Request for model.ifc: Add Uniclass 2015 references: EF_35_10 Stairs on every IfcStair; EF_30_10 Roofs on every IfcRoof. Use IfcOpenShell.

First a look at what the model holds.

```python
import ifcopenshell

model = ifcopenshell.open("model.ifc")
print(model.schema)
print("classifications:", [c.Name for c in model.by_type("IfcClassification")])
for ifc_class in ("IfcDoor", "IfcRoof", "IfcStair", "IfcWall", "IfcWindow"):
    print(ifc_class, len(model.by_type(ifc_class)))
```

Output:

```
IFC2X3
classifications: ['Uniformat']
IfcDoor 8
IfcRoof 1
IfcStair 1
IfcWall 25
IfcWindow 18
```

```python
import ifcopenshell
import ifcopenshell.api.classification

model = ifcopenshell.open("model.ifc")

# IFC2X3 requires Source and Edition and has no link from the project to the system.
system = model.create_entity("IfcClassification", Source="NBS", Edition="2015", Name="Uniclass 2015")

codes = {
    "IfcStair": ("EF_35_10", "Stairs"),
    "IfcRoof": ("EF_30_10", "Roofs"),
}
for ifc_class, (code, name) in codes.items():
    products = model.by_type(ifc_class)
    ifcopenshell.api.classification.add_reference(
        model, products=products, classification=system, identification=code, name=name
    )
    print(code, len(products))

model.write("model-out.ifc")
```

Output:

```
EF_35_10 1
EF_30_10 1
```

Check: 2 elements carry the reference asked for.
